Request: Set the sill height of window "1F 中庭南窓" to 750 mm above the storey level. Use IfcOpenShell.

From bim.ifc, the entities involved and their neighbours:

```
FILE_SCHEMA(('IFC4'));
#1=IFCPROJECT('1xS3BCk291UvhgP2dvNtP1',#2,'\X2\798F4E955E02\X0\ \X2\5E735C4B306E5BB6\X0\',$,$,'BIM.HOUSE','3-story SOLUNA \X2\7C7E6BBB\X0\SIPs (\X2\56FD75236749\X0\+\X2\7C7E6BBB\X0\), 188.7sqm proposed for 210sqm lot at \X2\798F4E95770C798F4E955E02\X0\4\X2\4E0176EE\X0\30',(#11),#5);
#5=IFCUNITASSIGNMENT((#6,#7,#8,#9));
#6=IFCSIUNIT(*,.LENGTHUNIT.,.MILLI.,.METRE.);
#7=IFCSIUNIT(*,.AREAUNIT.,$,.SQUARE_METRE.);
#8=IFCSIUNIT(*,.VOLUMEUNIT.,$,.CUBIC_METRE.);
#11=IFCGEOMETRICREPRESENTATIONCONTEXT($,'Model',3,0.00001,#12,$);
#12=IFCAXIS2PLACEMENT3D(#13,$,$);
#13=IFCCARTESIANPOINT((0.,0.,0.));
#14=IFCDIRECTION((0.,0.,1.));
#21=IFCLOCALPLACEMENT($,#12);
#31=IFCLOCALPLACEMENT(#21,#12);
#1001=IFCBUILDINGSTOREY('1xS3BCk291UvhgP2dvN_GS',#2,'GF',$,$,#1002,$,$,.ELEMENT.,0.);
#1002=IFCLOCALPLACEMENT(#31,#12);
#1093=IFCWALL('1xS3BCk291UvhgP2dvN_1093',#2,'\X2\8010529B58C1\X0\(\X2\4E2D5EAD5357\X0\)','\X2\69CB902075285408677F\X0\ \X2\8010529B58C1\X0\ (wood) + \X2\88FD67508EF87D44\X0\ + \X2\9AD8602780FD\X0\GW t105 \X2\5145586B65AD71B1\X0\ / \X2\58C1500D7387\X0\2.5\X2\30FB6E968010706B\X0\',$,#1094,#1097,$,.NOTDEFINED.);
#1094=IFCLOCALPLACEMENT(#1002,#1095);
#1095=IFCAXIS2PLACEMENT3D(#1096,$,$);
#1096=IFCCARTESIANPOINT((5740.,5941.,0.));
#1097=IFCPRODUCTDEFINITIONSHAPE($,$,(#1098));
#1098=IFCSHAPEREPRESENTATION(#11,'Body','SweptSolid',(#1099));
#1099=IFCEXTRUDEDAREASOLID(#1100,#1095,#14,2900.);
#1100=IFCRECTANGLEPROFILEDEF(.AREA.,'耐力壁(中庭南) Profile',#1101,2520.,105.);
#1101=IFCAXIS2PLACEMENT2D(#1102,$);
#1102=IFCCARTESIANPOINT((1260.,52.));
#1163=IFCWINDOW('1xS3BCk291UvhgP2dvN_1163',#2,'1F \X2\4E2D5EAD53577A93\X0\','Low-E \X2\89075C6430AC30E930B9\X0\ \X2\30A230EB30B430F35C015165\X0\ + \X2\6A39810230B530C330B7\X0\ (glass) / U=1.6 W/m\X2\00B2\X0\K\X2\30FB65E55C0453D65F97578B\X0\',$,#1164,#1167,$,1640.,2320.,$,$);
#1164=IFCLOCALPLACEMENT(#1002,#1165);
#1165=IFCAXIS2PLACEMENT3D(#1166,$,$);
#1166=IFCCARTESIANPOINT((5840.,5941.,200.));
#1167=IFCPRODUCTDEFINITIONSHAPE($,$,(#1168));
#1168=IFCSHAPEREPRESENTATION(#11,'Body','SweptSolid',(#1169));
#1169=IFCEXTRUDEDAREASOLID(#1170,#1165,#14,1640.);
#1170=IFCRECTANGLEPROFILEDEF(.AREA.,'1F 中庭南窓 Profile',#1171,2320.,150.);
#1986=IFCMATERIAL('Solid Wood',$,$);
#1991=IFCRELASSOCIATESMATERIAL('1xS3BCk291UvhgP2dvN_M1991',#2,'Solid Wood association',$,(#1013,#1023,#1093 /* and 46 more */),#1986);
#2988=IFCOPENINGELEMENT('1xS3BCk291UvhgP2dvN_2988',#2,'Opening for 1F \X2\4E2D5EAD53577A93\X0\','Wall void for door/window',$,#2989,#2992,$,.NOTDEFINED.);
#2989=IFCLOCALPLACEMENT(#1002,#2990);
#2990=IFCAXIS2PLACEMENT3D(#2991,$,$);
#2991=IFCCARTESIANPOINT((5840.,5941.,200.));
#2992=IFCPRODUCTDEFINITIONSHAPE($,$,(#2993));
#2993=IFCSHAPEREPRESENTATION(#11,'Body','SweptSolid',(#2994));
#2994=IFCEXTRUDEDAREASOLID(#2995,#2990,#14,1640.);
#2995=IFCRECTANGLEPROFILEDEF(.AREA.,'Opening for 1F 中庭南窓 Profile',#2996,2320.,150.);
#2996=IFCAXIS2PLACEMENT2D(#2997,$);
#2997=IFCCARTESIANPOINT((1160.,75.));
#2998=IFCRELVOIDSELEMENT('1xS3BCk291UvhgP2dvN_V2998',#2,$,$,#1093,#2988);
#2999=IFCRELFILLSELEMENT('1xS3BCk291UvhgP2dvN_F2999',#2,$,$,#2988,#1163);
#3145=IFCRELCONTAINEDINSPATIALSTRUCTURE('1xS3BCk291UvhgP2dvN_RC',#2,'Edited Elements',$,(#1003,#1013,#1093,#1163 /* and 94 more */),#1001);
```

```python
import numpy as np
import ifcopenshell
import ifcopenshell.api.geometry
import ifcopenshell.geom
import ifcopenshell.util.element
import ifcopenshell.util.placement
import ifcopenshell.util.shape
import ifcopenshell.util.unit

model = ifcopenshell.open("bim.ifc")
unit_scale = ifcopenshell.util.unit.calculate_unit_scale(model)

window = model.by_guid("1xS3BCk291UvhgP2dvN_1163")
opening = window.FillsVoids[0].RelatingOpeningElement
storey = ifcopenshell.util.element.get_container(window, ifc_class="IfcBuildingStorey")
level = ifcopenshell.util.placement.get_local_placement(storey.ObjectPlacement)[2, 3]

# The opening's origin need not be at the sill, so measure its lowest point.
shape = ifcopenshell.geom.create_shape(ifcopenshell.geom.settings(), opening)
bottom = ifcopenshell.util.shape.get_shape_bottom_elevation(shape, shape.geometry) / unit_scale
dz = level + 750.0 - bottom

shift = np.array([0.0, 0.0, dz])
# The window is not placed relative to its opening, so move both.
for product in (opening, window):
    matrix = ifcopenshell.util.placement.get_local_placement(product.ObjectPlacement)
    matrix[:3, 3] += shift
    ifcopenshell.api.geometry.edit_object_placement(model, product=product, matrix=matrix, is_si=False)

print(f"moved by {dz * unit_scale:+.3f} m")

model.write("bim_edited.ifc")
```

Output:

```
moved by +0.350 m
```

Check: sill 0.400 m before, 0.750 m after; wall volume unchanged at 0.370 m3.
